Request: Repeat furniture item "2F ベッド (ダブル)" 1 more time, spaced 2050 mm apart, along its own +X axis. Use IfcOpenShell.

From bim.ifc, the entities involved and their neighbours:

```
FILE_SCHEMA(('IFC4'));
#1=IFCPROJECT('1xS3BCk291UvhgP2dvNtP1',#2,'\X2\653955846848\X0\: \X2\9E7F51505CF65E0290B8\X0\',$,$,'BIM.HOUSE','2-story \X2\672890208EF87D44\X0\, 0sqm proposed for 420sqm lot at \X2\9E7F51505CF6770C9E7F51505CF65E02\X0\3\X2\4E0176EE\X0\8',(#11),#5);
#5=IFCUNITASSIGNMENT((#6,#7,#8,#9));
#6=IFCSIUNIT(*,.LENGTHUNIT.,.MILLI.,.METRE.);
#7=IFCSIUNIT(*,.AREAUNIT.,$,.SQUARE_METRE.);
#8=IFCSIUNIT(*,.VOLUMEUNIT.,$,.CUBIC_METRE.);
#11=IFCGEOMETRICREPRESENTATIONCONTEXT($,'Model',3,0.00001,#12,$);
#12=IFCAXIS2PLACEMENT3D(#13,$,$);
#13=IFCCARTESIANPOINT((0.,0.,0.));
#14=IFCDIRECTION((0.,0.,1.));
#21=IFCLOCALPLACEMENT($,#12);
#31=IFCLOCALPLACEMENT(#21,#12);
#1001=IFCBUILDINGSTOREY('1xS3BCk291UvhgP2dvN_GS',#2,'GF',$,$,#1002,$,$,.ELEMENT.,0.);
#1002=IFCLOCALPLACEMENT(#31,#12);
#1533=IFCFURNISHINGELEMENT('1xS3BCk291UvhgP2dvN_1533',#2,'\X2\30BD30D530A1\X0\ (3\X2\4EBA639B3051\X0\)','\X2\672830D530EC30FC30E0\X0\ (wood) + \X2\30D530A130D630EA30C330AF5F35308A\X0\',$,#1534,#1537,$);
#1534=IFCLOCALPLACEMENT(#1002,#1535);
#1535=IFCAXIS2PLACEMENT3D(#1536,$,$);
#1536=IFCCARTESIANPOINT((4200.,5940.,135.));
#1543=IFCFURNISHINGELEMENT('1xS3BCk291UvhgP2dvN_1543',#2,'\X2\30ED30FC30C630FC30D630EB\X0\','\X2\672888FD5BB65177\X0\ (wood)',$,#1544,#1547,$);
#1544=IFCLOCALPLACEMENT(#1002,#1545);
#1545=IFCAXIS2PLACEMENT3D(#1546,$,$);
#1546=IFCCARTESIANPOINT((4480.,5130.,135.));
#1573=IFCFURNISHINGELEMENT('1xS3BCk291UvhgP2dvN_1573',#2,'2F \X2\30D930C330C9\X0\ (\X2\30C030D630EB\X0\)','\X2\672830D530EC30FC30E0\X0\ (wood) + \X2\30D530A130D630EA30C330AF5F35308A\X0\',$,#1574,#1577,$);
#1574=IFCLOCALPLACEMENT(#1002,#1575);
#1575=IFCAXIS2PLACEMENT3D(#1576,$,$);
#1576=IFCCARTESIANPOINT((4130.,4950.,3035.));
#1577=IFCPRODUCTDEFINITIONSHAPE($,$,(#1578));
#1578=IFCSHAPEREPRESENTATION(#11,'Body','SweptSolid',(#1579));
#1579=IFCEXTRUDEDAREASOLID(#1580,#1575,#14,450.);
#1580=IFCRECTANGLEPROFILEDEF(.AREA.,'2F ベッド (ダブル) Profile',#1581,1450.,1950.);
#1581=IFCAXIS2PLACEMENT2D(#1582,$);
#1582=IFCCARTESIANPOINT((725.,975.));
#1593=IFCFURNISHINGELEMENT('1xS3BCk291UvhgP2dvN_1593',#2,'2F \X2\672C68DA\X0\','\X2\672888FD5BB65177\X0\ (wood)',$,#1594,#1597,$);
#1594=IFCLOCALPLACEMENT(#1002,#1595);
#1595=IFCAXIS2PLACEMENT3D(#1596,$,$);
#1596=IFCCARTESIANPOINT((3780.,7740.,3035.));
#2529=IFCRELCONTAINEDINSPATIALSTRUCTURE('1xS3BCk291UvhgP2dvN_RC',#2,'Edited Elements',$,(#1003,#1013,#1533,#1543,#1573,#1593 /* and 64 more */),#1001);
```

```python
import ifcopenshell
import ifcopenshell.api.geometry
import ifcopenshell.api.root
import ifcopenshell.util.element
import ifcopenshell.util.placement
import ifcopenshell.util.unit

model = ifcopenshell.open("bim.ifc")
unit_scale = ifcopenshell.util.unit.calculate_unit_scale(model)


def reuse_history(source, copy):
    """copy_class also copies each property set's owner history, people and application; keep the originals."""
    for rel in copy.IsDefinedBy:
        if rel.is_a("IfcRelDefinesByProperties") and (history := rel.RelatingPropertyDefinition.OwnerHistory):
            rel.RelatingPropertyDefinition.OwnerHistory = source.OwnerHistory
            ifcopenshell.util.element.remove_deep2(model, history)


source = model.by_guid("1xS3BCk291UvhgP2dvN_1573")
base = ifcopenshell.util.placement.get_local_placement(source.ObjectPlacement)
step = base[:3, 0] * 2.05 / unit_scale

for i in range(1, 2):
    copy = ifcopenshell.api.root.copy_class(model, product=source)
    copy.Representation = ifcopenshell.util.element.copy_deep(
        model, source.Representation, exclude=["IfcGeometricRepresentationContext", "IfcRepresentationMap"]
    )
    reuse_history(source, copy)
    matrix = base.copy()
    matrix[:3, 3] += i * step
    print("added at", matrix[:3, 3].round(3) + 0.0)
    ifcopenshell.api.geometry.edit_object_placement(model, product=copy, matrix=matrix, is_si=False)

model.write("bim_edited.ifc")
```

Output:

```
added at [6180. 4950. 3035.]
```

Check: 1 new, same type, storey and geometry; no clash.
